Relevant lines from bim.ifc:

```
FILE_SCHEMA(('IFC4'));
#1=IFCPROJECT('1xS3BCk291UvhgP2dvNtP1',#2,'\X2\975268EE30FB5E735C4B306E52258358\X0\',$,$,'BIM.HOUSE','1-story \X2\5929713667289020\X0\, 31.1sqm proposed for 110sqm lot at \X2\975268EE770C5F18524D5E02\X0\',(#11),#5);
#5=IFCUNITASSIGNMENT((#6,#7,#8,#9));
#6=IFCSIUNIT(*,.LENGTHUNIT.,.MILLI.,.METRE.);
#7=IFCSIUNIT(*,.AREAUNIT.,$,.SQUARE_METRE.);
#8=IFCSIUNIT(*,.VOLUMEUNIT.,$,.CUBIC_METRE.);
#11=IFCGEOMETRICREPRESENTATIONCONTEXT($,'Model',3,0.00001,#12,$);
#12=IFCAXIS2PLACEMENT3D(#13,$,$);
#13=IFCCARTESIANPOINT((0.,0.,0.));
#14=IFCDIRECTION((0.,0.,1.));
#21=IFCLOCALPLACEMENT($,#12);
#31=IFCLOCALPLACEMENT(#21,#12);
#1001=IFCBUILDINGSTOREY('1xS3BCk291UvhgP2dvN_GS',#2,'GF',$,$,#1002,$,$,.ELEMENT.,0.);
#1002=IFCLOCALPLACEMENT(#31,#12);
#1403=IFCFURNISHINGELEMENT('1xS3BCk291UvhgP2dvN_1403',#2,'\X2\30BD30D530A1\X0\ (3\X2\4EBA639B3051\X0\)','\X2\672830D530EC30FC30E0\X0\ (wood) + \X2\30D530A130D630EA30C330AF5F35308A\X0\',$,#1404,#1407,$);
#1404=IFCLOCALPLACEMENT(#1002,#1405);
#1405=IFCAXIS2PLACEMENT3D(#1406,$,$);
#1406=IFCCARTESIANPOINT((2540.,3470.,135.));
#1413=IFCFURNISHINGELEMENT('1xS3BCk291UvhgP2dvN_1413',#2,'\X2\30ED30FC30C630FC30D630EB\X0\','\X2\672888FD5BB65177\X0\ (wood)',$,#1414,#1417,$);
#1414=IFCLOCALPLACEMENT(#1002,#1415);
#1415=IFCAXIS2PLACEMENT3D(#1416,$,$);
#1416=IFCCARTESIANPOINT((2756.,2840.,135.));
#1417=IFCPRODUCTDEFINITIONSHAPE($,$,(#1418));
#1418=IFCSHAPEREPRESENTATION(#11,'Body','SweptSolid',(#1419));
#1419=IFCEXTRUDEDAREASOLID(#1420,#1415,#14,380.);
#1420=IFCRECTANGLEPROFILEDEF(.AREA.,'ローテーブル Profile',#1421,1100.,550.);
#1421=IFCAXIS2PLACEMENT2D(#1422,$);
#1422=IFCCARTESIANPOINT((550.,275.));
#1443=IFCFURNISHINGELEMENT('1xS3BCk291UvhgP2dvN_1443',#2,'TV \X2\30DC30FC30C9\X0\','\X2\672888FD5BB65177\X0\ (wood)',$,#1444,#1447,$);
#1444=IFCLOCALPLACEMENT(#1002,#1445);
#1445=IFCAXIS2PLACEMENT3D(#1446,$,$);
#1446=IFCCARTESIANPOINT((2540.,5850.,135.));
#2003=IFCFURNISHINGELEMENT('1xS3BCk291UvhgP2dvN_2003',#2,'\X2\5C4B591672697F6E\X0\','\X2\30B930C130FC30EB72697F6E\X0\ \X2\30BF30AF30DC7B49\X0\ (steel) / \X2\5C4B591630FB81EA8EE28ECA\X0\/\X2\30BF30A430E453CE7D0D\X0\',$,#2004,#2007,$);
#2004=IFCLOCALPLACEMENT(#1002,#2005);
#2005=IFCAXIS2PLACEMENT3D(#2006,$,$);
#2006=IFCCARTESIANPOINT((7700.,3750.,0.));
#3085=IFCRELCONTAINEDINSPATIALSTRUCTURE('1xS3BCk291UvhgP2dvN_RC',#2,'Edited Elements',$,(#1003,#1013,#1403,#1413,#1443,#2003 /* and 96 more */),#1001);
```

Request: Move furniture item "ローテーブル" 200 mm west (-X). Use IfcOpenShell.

```python
import ifcopenshell
import ifcopenshell.api.geometry
import ifcopenshell.util.placement

model = ifcopenshell.open("bim.ifc")

item = model.by_guid("1xS3BCk291UvhgP2dvN_1413")
matrix = ifcopenshell.util.placement.get_local_placement(item.ObjectPlacement)
matrix[0, 3] -= 200.0
ifcopenshell.api.geometry.edit_object_placement(model, product=item, matrix=matrix, is_si=False)

print(ifcopenshell.util.placement.get_local_placement(item.ObjectPlacement).round(3) + 0.0)

model.write("bim_v2.ifc")
```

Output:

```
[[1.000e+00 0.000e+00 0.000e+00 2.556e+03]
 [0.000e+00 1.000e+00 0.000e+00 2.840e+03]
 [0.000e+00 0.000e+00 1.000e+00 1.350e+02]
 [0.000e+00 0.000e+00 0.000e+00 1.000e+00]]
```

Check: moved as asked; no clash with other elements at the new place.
